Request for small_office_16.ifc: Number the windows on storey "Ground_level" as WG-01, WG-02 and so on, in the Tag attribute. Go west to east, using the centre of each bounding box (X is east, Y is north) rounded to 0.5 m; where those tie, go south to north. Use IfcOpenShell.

First a look at what the model holds.

```python
import ifcopenshell
import ifcopenshell.util.element
import ifcopenshell.util.placement

model = ifcopenshell.open("small_office_16.ifc")
print(model.schema)
storey = next(s for s in model.by_type("IfcBuildingStorey") if s.Name == "Ground_level")
windows = [e for e in ifcopenshell.util.element.get_decomposition(storey) if e.is_a("IfcWindow")]
for e in sorted(windows, key=lambda e: e.id()):
    origin = ifcopenshell.util.placement.get_local_placement(e.ObjectPlacement)[:3, 3]
    print(e.id(), e.Tag, e.Name, origin.round(2) + 0.0, sep=" | ")
```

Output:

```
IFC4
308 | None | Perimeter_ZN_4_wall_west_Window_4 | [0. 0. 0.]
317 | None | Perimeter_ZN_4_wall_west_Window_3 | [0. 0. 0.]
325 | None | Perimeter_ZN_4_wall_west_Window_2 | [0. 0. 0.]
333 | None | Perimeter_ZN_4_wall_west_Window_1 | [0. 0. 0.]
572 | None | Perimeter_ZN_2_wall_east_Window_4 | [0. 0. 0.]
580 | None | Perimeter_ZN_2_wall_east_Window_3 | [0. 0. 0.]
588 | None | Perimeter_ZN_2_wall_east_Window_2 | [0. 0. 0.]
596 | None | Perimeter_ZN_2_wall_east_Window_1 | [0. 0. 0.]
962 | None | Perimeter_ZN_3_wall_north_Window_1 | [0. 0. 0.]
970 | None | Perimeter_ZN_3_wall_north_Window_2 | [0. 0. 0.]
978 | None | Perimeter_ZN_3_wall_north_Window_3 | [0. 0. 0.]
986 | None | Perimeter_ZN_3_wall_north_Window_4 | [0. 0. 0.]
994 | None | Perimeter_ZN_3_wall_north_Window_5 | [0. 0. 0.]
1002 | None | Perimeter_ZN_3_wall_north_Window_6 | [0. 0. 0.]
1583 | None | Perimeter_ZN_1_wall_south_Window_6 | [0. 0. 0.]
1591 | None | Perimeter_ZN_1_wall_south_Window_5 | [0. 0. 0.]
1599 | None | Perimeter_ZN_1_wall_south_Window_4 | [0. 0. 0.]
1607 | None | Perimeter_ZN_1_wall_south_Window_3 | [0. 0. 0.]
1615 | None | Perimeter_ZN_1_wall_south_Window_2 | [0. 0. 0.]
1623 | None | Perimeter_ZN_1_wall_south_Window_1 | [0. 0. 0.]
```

```python
import ifcopenshell
import ifcopenshell.geom
import ifcopenshell.util.element
import ifcopenshell.util.shape

model = ifcopenshell.open("small_office_16.ifc")
settings = ifcopenshell.geom.settings()
settings.set("use-world-coords", True)


def centre(element):
    shape = ifcopenshell.geom.create_shape(settings, element)
    return ifcopenshell.util.shape.get_bbox_centroid(shape.geometry)


storey = next(s for s in model.by_type("IfcBuildingStorey") if s.Name == "Ground_level")
windows = [e for e in ifcopenshell.util.element.get_decomposition(storey) if e.is_a("IfcWindow")]

# Insertion points can sit at a corner or the storey origin, so sort by the geometry (in metres).
centres = {e: centre(e) for e in windows}
windows.sort(key=lambda e: (round(centres[e][0] / 0.5), centres[e][1]))

for i, e in enumerate(windows, start=1):
    number = f"WG-{i:02d}"
    e.Tag = number
    print(e.id(), number)

model.write("small_office_16_rev.ifc")
```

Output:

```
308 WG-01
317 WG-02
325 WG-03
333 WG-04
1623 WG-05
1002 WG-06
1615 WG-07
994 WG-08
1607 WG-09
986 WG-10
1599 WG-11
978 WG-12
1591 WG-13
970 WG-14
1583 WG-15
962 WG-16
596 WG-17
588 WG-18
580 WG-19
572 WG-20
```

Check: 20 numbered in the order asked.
